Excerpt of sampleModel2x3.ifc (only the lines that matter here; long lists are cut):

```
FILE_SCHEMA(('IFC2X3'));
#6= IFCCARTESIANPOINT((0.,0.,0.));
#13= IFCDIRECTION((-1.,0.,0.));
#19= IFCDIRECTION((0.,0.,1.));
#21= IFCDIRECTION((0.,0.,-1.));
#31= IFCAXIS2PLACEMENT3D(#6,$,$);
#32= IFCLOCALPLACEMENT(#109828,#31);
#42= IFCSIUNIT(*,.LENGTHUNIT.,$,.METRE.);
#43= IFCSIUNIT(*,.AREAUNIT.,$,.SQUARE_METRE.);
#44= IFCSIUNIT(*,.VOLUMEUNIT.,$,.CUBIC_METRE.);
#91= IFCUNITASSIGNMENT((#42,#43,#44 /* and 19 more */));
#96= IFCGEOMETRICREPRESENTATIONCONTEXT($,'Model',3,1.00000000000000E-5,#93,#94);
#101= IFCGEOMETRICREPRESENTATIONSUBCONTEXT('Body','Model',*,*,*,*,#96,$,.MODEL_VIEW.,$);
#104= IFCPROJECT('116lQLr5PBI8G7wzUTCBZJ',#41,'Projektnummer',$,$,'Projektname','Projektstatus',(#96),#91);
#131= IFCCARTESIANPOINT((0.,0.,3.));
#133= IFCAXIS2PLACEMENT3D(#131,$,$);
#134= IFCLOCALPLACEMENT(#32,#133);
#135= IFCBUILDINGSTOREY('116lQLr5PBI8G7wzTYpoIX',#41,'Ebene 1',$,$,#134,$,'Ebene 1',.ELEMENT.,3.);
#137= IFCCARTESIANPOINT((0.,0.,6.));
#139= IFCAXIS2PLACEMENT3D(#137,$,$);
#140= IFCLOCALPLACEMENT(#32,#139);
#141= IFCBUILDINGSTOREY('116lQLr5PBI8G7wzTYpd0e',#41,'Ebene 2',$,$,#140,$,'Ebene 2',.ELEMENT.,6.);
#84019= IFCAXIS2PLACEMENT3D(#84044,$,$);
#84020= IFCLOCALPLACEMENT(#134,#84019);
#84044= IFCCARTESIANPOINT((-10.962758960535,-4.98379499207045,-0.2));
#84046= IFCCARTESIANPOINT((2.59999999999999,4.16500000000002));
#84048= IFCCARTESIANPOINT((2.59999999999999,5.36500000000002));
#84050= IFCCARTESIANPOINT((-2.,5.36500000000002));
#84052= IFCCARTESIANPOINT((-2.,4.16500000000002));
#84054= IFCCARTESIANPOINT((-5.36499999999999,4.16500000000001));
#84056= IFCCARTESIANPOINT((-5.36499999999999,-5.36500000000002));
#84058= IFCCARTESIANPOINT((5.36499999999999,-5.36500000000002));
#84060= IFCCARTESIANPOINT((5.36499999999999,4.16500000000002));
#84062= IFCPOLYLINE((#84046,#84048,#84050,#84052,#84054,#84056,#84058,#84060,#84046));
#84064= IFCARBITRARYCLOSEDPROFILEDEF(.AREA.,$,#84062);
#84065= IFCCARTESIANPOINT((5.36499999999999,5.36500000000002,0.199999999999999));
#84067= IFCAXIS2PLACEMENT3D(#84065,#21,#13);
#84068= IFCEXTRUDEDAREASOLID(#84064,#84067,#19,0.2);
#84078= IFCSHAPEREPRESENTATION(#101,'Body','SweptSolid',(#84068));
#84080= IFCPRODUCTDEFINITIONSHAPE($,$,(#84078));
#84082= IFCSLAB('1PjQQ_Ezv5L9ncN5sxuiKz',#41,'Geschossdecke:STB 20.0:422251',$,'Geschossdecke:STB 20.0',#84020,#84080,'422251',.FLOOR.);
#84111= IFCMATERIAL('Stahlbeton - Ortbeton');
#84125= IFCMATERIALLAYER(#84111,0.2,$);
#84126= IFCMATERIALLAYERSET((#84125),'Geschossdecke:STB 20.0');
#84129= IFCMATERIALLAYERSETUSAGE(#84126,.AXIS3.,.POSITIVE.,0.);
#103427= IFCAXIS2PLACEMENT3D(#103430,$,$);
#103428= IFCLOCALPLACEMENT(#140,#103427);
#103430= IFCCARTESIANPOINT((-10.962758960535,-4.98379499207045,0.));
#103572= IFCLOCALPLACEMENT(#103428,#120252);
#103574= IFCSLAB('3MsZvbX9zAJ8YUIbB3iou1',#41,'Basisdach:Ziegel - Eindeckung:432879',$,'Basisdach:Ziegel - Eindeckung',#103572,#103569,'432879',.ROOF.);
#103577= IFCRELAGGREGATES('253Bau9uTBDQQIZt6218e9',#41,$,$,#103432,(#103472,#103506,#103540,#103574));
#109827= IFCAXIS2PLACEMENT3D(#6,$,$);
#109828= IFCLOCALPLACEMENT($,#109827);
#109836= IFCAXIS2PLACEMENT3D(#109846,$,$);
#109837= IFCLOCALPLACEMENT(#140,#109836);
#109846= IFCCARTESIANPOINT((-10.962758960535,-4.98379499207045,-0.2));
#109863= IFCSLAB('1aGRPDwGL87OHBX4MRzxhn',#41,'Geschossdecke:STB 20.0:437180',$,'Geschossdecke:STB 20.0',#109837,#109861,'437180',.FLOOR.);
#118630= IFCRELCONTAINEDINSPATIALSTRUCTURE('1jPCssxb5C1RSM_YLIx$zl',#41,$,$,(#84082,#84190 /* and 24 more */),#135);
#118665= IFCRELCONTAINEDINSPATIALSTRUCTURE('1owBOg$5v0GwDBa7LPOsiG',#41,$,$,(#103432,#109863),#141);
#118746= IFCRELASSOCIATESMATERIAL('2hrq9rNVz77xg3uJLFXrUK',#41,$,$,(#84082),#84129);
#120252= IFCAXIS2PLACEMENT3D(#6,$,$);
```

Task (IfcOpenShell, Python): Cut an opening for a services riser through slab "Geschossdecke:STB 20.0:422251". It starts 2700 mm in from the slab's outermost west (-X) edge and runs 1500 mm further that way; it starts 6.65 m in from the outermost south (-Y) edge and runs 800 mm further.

```python
import numpy as np
import ifcopenshell
import ifcopenshell.api.feature
import ifcopenshell.api.geometry
import ifcopenshell.api.root
import ifcopenshell.geom
import ifcopenshell.util.placement
import ifcopenshell.util.representation
import ifcopenshell.util.shape
import ifcopenshell.util.unit

model = ifcopenshell.open("sampleModel2x3.ifc")
unit_scale = ifcopenshell.util.unit.calculate_unit_scale(model)
settings = ifcopenshell.geom.settings()


def volume(element):
    """Net volume in cubic metres, openings subtracted."""
    shape = ifcopenshell.geom.create_shape(settings, element)
    return ifcopenshell.util.shape.get_volume(shape.geometry)


slab = model.by_guid("1PjQQ_Ezv5L9ncN5sxuiKz")
before = volume(slab)

# Extent in the slab's own axes, in metres. The edges named are its -X and -Y sides.
slab_shape = ifcopenshell.geom.create_shape(settings, slab)
vertices = ifcopenshell.util.shape.get_vertices(slab_shape.geometry)
x_min, y_min, bottom = vertices.min(axis=0)
top = vertices[:, 2].max()

opening = ifcopenshell.api.root.create_entity(model, ifc_class="IfcOpeningElement", name="Services riser opening")
context = ifcopenshell.util.representation.get_context(model, "Model", "Body", "MODEL_VIEW")
width, depth = 1.5, 0.8
outline = [(0.0, 0.0), (width, 0.0), (width, depth), (0.0, depth), (0.0, 0.0)]
# Overshoot both faces by 50 mm so the cut is clean.
shape = ifcopenshell.api.geometry.add_slab_representation(
    model, context=context, depth=top - bottom + 0.1, polyline=outline
)
ifcopenshell.api.geometry.assign_representation(model, product=opening, representation=shape)

matrix = ifcopenshell.util.placement.get_local_placement(slab.ObjectPlacement)
matrix[:, 3] = matrix @ np.append(np.array([x_min + 2.7, y_min + 6.65, bottom - 0.05]) / unit_scale, 1.0)
ifcopenshell.api.geometry.edit_object_placement(model, product=opening, matrix=matrix, is_si=False)
ifcopenshell.api.feature.add_feature(model, feature=opening, element=slab)

after = volume(slab)

print(f"slab volume {before:.3f} -> {after:.3f} m3")

model.write("sampleModel2x3_updated.ifc")
```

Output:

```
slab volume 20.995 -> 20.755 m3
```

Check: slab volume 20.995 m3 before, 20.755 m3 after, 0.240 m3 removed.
